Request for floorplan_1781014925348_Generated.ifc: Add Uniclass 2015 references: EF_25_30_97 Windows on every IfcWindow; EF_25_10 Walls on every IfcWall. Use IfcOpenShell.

First a look at what the model holds.

```python
import ifcopenshell

model = ifcopenshell.open("floorplan_1781014925348_Generated.ifc")
print(model.schema)
print("classifications:", [c.Name for c in model.by_type("IfcClassification")])
for ifc_class in ("IfcDoor", "IfcRoof", "IfcStair", "IfcWall", "IfcWindow"):
    print(ifc_class, len(model.by_type(ifc_class)))
```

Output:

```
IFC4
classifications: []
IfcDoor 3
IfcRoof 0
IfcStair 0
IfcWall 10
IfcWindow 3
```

```python
import ifcopenshell
import ifcopenshell.api.classification

model = ifcopenshell.open("floorplan_1781014925348_Generated.ifc")

system = ifcopenshell.api.classification.add_classification(model, classification="Uniclass 2015")

codes = {
    "IfcWindow": ("EF_25_30_97", "Windows"),
    "IfcWall": ("EF_25_10", "Walls"),
}
for ifc_class, (code, name) in codes.items():
    products = model.by_type(ifc_class)
    ifcopenshell.api.classification.add_reference(
        model, products=products, classification=system, identification=code, name=name
    )
    print(code, len(products))

model.write("floorplan_1781014925348_Generated_updated.ifc")
```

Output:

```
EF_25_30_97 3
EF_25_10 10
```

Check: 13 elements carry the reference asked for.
